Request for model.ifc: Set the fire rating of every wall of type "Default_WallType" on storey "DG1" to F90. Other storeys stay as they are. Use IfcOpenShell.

First a look at what the model holds.

```python
import ifcopenshell
import ifcopenshell.util.element

model = ifcopenshell.open("model.ifc")
print(model.schema)
storey = next(s for s in model.by_type("IfcBuildingStorey") if s.Name == "DG1")
walls = [e for e in ifcopenshell.util.element.get_decomposition(storey) if e.is_a("IfcWall")]
seen = {}
for e in walls:
    element_type = ifcopenshell.util.element.get_type(e)
    key = (element_type.Name if element_type != e and element_type else None, ifcopenshell.util.element.get_pset(e, "Pset_WallCommon", "FireRating"))
    seen[key] = seen.get(key, 0) + 1
for (name, value), count in sorted(seen.items(), key=str):
    print(count, "x", name, "|", value)
```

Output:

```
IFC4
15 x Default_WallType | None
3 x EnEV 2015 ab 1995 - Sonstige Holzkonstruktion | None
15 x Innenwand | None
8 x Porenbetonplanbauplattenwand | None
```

```python
import ifcopenshell
import ifcopenshell.api.pset
import ifcopenshell.util.element

model = ifcopenshell.open("model.ifc")

storey = next(s for s in model.by_type("IfcBuildingStorey") if s.Name == "DG1")
walls = [e for e in ifcopenshell.util.element.get_decomposition(storey) if e.is_a("IfcWall")]

count = 0
for e in walls:
    element_type = ifcopenshell.util.element.get_type(e)
    if element_type in (None, e) or element_type.Name != "Default_WallType":
        continue
    # add_pset returns the element's existing set when there is one.
    pset = ifcopenshell.api.pset.add_pset(model, product=e, name="Pset_WallCommon")
    ifcopenshell.api.pset.edit_pset(model, pset=pset, properties={"FireRating": "F90"})
    count += 1

print(count, "walls updated")

model.write("model_rev.ifc")
```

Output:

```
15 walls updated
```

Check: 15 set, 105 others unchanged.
